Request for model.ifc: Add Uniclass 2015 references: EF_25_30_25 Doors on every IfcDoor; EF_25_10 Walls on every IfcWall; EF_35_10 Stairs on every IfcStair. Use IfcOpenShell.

First a look at what the model holds.

```python
import ifcopenshell

model = ifcopenshell.open("model.ifc")
print(model.schema)
print("classifications:", [c.Name for c in model.by_type("IfcClassification")])
for ifc_class in ("IfcDoor", "IfcRoof", "IfcStair", "IfcWall", "IfcWindow"):
    print(ifc_class, len(model.by_type(ifc_class)))
```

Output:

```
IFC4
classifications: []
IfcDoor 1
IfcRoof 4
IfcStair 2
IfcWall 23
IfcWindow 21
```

```python
import ifcopenshell
import ifcopenshell.api.classification

model = ifcopenshell.open("model.ifc")

system = ifcopenshell.api.classification.add_classification(model, classification="Uniclass 2015")

codes = {
    "IfcDoor": ("EF_25_30_25", "Doors"),
    "IfcWall": ("EF_25_10", "Walls"),
    "IfcStair": ("EF_35_10", "Stairs"),
}
for ifc_class, (code, name) in codes.items():
    products = model.by_type(ifc_class)
    ifcopenshell.api.classification.add_reference(
        model, products=products, classification=system, identification=code, name=name
    )
    print(code, len(products))

model.write("model_rev.ifc")
```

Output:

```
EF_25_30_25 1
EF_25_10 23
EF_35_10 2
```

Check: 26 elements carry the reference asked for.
